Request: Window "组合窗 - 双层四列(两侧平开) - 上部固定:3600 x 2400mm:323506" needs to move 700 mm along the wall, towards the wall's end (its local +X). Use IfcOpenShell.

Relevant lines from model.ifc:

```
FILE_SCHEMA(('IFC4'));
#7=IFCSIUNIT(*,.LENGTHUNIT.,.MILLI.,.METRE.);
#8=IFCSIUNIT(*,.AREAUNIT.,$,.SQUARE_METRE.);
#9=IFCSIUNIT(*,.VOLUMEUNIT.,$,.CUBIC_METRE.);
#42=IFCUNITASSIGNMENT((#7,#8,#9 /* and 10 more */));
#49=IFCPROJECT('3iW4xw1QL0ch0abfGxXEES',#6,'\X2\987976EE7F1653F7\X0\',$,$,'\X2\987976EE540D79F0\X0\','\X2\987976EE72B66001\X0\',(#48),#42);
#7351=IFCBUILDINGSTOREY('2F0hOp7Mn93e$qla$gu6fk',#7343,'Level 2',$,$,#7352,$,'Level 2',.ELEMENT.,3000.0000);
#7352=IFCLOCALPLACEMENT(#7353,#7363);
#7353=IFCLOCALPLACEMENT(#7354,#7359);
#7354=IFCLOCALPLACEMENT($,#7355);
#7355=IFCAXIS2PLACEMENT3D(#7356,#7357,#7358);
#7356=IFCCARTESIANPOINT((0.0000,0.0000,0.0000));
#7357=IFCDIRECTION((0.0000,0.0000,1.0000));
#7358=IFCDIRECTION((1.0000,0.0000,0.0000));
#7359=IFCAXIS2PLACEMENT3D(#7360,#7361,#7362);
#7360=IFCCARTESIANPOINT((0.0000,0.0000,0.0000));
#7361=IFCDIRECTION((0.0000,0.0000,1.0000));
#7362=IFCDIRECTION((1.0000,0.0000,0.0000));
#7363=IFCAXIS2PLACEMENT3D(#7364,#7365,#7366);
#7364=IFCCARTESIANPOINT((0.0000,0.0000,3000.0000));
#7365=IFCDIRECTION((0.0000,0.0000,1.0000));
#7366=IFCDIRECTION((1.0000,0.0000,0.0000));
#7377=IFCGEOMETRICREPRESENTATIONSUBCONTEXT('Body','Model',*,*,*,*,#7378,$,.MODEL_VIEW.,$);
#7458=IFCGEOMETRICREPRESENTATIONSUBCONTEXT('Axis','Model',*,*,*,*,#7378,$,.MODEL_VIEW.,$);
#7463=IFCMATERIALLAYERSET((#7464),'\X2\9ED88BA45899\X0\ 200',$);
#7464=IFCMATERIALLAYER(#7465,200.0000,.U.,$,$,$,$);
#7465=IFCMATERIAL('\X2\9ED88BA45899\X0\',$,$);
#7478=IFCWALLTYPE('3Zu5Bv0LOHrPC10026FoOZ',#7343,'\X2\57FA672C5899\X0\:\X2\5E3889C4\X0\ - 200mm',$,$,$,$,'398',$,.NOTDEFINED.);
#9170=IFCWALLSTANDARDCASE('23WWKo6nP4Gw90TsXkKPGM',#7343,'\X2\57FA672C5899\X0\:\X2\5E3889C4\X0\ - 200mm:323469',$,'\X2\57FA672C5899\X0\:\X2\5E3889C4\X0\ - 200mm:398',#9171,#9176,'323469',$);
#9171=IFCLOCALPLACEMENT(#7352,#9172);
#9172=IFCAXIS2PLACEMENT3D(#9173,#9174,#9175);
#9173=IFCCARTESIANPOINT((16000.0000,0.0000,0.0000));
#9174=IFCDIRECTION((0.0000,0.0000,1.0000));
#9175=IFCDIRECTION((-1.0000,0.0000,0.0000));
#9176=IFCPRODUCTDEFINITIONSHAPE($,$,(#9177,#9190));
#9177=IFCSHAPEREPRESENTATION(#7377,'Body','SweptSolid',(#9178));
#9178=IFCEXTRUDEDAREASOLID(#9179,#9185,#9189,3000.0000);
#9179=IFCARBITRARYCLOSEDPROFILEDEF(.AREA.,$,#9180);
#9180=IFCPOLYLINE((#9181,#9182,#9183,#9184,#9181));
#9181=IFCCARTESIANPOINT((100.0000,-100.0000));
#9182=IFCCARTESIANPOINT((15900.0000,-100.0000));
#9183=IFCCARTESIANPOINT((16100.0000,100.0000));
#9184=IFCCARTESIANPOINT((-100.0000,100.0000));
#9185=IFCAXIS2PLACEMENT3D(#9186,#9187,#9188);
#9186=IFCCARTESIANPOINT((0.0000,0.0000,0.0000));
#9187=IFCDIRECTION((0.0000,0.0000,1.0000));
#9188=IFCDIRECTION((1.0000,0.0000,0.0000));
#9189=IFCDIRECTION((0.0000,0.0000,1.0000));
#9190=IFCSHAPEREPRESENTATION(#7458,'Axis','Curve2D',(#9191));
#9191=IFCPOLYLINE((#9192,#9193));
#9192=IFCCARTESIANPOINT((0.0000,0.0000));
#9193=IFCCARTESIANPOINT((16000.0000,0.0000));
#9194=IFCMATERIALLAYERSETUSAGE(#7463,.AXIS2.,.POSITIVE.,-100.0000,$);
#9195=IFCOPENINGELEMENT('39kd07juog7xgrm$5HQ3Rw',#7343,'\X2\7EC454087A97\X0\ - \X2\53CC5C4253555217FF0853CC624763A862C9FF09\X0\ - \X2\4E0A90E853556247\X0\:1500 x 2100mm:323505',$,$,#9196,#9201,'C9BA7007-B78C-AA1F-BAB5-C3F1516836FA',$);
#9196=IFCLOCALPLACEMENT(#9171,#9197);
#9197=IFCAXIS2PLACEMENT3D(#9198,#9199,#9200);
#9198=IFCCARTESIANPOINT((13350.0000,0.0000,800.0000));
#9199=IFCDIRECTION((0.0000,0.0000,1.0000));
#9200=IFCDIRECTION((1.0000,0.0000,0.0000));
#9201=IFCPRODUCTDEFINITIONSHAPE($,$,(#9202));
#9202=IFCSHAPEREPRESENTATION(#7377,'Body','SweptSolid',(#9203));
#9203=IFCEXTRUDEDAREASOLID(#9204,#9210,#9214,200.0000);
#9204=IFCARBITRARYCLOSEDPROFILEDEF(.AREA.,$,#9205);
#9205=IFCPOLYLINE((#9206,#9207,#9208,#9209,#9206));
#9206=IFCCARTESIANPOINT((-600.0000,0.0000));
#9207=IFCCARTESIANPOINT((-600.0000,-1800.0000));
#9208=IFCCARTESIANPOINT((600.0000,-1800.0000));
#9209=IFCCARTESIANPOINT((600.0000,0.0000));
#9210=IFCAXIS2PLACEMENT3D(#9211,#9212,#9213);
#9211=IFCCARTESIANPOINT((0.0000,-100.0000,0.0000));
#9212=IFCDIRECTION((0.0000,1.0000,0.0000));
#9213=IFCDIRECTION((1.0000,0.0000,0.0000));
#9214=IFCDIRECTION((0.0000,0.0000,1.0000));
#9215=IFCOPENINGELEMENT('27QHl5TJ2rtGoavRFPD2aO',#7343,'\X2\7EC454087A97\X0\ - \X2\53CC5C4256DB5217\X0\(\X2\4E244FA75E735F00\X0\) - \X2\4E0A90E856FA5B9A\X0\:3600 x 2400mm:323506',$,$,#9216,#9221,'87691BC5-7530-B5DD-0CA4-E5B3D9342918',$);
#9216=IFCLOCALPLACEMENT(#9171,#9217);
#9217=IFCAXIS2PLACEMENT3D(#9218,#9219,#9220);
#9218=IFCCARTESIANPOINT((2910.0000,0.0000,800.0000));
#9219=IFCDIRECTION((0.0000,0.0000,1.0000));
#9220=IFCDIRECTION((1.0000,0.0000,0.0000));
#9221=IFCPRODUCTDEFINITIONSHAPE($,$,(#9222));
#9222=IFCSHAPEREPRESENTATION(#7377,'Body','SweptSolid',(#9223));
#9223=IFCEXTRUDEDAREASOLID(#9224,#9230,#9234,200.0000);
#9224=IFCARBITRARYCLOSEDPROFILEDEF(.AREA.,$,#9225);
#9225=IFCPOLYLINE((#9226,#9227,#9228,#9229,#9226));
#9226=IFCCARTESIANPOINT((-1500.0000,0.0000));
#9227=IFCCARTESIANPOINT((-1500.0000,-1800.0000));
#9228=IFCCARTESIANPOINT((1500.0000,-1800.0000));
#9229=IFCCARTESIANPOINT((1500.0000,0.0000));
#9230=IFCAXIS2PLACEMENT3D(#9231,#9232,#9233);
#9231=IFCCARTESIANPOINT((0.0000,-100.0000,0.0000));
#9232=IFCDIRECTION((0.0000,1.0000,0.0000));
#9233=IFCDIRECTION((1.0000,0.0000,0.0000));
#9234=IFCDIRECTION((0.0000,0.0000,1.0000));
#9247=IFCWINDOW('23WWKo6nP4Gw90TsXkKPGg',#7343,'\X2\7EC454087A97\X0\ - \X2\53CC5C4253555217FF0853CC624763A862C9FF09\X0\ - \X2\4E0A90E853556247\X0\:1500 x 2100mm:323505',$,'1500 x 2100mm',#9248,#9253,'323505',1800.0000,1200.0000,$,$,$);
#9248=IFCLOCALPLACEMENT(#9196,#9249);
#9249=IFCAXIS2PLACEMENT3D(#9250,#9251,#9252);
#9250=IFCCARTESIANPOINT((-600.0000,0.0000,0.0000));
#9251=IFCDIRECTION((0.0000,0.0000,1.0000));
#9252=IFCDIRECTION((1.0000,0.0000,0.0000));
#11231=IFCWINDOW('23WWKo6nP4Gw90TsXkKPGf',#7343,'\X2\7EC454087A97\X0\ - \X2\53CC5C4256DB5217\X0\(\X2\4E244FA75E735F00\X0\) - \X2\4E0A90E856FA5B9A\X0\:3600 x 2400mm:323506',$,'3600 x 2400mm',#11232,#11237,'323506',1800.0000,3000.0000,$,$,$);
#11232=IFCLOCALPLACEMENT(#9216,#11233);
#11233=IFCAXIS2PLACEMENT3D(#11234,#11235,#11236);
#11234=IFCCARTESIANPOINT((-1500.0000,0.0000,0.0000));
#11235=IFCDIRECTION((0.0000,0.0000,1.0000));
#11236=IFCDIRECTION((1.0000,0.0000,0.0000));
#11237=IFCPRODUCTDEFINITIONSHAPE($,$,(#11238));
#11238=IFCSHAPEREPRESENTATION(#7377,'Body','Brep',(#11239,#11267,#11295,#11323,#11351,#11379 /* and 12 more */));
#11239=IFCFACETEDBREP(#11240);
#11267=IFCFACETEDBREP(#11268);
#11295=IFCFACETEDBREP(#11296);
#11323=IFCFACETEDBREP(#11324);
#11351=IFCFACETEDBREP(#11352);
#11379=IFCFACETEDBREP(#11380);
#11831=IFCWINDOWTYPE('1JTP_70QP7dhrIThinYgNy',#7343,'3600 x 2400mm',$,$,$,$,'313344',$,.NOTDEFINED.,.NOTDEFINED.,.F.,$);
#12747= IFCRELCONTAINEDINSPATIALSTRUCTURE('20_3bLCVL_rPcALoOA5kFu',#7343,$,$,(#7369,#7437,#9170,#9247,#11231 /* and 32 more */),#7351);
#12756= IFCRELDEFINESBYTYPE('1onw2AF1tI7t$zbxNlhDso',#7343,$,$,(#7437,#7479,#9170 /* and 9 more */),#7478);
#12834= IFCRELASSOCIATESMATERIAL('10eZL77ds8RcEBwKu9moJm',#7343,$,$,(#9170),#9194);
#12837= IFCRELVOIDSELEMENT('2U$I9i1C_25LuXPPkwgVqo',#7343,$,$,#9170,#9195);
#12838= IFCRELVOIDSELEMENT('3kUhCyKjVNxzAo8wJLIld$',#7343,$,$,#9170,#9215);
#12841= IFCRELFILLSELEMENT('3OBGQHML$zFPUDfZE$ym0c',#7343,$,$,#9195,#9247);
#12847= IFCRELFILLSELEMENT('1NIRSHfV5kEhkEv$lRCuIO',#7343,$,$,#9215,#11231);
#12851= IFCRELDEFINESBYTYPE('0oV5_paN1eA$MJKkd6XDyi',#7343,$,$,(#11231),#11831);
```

```python
import ifcopenshell
import ifcopenshell.api.geometry
import ifcopenshell.util.placement
import ifcopenshell.util.unit

model = ifcopenshell.open("model.ifc")
unit_scale = ifcopenshell.util.unit.calculate_unit_scale(model)

window = model.by_id(11231)
opening = window.FillsVoids[0].RelatingOpeningElement
wall = opening.VoidsElements[0].RelatingBuildingElement

wall_matrix = ifcopenshell.util.placement.get_local_placement(wall.ObjectPlacement)
shift = wall_matrix[:3, 0] * 0.7 / unit_scale
before = ifcopenshell.util.placement.get_local_placement(window.ObjectPlacement)[:3, 3].copy()

# The window is placed relative to its opening, so it follows when the opening moves.
matrix = ifcopenshell.util.placement.get_local_placement(opening.ObjectPlacement)
matrix[:3, 3] += shift
ifcopenshell.api.geometry.edit_object_placement(
    model, product=opening, matrix=matrix, is_si=False, should_transform_children=True
)

after = ifcopenshell.util.placement.get_local_placement(window.ObjectPlacement)[:3, 3]
print("window moved by", (after - before).round(3) + 0.0)

model.write("model_rev.ifc")
```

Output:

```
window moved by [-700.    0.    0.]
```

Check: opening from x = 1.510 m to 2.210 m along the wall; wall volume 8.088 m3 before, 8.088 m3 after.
